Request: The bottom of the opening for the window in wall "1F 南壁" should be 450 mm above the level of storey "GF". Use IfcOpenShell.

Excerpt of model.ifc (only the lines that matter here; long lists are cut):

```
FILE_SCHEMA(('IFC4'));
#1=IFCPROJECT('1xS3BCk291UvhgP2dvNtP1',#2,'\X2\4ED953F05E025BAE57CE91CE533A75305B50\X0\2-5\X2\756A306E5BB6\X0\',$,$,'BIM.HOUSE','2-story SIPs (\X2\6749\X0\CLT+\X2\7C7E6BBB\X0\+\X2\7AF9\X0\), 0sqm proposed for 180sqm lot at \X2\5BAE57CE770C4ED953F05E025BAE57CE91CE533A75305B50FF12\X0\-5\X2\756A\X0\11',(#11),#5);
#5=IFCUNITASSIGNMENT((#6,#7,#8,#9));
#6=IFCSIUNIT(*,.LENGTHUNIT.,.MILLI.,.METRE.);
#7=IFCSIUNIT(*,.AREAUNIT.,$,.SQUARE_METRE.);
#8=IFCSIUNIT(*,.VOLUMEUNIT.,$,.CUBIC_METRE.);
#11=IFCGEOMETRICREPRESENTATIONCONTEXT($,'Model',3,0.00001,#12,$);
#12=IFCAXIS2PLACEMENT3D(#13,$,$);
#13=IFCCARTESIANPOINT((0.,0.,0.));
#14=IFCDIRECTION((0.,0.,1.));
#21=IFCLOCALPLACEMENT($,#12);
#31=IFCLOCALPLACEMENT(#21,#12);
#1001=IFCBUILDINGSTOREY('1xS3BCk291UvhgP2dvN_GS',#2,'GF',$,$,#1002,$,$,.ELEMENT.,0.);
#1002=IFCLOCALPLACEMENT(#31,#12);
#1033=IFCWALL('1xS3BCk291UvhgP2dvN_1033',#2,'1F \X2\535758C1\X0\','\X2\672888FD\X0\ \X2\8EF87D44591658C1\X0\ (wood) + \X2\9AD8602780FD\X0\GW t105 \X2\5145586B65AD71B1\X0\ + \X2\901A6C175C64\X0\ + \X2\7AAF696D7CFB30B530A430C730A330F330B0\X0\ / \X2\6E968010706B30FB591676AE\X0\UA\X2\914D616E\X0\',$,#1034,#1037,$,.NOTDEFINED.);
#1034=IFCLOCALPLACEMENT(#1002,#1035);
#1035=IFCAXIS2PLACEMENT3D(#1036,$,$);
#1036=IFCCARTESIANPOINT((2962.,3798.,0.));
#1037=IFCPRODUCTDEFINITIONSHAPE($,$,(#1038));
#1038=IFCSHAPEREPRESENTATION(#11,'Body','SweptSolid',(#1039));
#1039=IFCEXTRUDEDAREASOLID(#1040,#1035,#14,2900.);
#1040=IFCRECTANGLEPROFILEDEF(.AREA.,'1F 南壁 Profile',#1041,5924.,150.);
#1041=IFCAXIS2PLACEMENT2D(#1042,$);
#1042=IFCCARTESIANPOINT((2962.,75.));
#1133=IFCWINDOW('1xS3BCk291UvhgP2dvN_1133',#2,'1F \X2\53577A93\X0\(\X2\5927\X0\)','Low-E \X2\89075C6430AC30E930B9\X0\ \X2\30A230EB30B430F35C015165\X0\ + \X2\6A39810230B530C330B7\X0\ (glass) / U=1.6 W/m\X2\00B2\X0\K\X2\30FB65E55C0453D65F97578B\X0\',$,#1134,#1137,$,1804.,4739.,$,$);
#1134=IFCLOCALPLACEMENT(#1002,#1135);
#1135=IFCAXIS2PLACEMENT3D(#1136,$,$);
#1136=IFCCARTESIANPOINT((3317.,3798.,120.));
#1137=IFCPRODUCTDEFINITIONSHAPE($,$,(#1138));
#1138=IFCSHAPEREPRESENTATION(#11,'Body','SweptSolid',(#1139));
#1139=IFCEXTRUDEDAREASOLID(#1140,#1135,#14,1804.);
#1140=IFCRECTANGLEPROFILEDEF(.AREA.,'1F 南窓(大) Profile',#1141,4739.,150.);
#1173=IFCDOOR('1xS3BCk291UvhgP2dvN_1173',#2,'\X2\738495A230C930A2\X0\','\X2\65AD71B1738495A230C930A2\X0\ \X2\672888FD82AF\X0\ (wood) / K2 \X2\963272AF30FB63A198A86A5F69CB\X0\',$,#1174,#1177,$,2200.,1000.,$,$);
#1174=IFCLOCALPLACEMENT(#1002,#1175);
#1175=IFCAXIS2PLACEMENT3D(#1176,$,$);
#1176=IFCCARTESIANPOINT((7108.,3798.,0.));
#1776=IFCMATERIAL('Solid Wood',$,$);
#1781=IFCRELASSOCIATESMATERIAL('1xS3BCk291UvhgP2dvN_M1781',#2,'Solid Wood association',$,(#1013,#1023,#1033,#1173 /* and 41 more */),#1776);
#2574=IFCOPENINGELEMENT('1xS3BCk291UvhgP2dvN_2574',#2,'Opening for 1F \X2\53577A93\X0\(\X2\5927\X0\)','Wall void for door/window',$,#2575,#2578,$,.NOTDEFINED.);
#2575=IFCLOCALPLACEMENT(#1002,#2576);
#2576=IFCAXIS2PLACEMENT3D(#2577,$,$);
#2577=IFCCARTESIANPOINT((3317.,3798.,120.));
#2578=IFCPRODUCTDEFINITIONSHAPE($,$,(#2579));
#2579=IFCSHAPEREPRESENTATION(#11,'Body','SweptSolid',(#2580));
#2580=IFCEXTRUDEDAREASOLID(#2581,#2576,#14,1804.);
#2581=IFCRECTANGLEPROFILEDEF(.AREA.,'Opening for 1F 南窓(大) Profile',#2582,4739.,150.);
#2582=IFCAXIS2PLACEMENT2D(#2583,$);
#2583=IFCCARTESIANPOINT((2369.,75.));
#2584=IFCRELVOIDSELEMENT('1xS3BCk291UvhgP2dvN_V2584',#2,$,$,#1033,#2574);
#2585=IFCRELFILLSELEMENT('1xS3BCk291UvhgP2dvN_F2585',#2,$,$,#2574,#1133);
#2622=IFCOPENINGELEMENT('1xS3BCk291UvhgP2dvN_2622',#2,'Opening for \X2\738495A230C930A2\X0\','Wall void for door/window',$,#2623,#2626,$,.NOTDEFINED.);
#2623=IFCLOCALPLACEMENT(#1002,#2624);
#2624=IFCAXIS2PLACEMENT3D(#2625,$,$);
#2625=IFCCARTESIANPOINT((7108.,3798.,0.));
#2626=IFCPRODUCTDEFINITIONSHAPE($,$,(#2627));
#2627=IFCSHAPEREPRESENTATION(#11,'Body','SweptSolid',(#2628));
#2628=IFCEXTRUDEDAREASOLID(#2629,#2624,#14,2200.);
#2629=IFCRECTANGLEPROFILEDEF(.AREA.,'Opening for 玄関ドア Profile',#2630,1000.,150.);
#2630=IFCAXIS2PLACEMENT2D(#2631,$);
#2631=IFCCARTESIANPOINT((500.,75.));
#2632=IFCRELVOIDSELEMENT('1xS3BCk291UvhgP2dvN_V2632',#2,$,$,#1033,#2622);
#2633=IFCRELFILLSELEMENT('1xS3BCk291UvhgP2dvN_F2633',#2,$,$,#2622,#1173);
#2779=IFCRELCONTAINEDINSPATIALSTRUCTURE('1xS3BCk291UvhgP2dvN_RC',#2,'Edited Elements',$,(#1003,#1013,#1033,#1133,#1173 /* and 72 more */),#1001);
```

```python
import numpy as np
import ifcopenshell
import ifcopenshell.api.geometry
import ifcopenshell.geom
import ifcopenshell.util.element
import ifcopenshell.util.placement
import ifcopenshell.util.shape
import ifcopenshell.util.unit

model = ifcopenshell.open("model.ifc")
unit_scale = ifcopenshell.util.unit.calculate_unit_scale(model)

window = model.by_id(1133)
opening = window.FillsVoids[0].RelatingOpeningElement
storey = ifcopenshell.util.element.get_container(window, ifc_class="IfcBuildingStorey")
level = ifcopenshell.util.placement.get_local_placement(storey.ObjectPlacement)[2, 3]

# The opening's origin need not be at the sill, so measure its lowest point.
shape = ifcopenshell.geom.create_shape(ifcopenshell.geom.settings(), opening)
bottom = ifcopenshell.util.shape.get_shape_bottom_elevation(shape, shape.geometry) / unit_scale
dz = level + 450.0 - bottom

shift = np.array([0.0, 0.0, dz])
# The window is not placed relative to its opening, so move both.
for product in (opening, window):
    matrix = ifcopenshell.util.placement.get_local_placement(product.ObjectPlacement)
    matrix[:3, 3] += shift
    ifcopenshell.api.geometry.edit_object_placement(model, product=product, matrix=matrix, is_si=False)

print(f"moved by {dz * unit_scale:+.3f} m")

model.write("model_updated.ifc")
```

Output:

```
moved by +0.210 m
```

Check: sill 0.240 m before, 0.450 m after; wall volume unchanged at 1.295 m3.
